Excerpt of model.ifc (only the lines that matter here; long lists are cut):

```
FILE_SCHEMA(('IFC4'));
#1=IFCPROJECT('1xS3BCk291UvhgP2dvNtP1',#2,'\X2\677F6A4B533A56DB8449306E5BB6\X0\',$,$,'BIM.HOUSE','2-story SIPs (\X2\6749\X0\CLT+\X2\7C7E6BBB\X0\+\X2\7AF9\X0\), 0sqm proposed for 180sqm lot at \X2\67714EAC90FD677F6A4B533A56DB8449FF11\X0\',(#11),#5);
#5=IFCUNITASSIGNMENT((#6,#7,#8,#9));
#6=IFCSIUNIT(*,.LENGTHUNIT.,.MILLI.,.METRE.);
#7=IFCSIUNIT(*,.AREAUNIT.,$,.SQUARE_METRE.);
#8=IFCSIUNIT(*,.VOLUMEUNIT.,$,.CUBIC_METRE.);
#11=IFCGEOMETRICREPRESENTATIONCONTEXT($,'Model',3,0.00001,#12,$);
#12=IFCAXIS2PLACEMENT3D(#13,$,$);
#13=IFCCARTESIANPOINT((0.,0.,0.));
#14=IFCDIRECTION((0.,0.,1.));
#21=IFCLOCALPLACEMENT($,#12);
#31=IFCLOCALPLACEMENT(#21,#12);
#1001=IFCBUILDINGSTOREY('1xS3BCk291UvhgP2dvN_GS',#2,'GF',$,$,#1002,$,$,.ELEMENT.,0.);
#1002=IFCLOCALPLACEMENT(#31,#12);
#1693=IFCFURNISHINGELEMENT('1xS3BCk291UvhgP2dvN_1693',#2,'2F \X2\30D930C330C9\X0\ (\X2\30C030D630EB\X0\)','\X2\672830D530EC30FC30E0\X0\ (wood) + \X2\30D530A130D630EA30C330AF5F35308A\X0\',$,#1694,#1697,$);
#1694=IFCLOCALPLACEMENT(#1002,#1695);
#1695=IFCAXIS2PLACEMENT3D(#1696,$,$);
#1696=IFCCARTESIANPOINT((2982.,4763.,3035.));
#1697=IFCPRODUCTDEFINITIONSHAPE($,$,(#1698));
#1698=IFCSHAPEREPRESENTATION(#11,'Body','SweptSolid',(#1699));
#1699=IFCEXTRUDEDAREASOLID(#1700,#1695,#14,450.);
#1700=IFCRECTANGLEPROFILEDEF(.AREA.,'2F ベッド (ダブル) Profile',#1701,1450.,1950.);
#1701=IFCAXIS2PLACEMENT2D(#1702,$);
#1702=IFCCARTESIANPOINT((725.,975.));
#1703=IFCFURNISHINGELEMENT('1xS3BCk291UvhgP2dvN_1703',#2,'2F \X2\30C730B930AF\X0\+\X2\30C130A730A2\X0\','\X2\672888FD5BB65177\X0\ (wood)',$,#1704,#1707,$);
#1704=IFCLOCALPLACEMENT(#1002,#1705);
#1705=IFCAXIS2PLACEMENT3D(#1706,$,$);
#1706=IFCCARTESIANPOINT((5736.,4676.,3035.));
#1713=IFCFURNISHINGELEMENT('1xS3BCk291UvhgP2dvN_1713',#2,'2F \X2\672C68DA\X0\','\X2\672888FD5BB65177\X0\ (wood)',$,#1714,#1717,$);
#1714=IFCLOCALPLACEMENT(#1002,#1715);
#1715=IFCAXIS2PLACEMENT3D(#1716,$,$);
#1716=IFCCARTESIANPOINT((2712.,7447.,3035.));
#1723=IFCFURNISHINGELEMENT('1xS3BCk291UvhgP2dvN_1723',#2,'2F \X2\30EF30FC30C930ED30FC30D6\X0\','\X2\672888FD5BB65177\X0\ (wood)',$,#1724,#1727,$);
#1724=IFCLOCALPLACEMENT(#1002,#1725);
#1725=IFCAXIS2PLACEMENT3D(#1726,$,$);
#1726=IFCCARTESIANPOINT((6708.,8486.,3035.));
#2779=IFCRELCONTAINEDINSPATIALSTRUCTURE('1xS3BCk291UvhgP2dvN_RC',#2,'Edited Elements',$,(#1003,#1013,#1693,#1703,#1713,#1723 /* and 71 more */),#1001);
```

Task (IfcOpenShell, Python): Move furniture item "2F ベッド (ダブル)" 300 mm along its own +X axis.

```python
import ifcopenshell
import ifcopenshell.api.geometry
import ifcopenshell.util.placement
import ifcopenshell.util.unit

model = ifcopenshell.open("model.ifc")
unit_scale = ifcopenshell.util.unit.calculate_unit_scale(model)

item = model.by_guid("1xS3BCk291UvhgP2dvN_1693")
matrix = ifcopenshell.util.placement.get_local_placement(item.ObjectPlacement)
matrix[:3, 3] += matrix[:3, 0] * 0.3 / unit_scale
ifcopenshell.api.geometry.edit_object_placement(model, product=item, matrix=matrix, is_si=False)

print(ifcopenshell.util.placement.get_local_placement(item.ObjectPlacement).round(3) + 0.0)

model.write("model_edited.ifc")
```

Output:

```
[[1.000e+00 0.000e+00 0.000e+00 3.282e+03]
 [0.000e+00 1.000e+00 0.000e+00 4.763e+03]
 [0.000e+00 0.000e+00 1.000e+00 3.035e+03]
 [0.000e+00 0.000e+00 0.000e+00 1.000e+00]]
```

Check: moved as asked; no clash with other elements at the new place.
